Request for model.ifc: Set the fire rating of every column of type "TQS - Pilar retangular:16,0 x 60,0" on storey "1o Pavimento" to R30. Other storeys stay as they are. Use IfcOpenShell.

First a look at what the model holds.

```python
import ifcopenshell
import ifcopenshell.util.element

model = ifcopenshell.open("model.ifc")
print(model.schema)
storey = next(s for s in model.by_type("IfcBuildingStorey") if s.Name == "1o Pavimento")
columns = [e for e in ifcopenshell.util.element.get_decomposition(storey) if e.is_a("IfcColumn")]
seen = {}
for e in columns:
    element_type = ifcopenshell.util.element.get_type(e)
    key = (element_type.Name if element_type != e and element_type else None, ifcopenshell.util.element.get_pset(e, "Pset_ColumnCommon", "FireRating"))
    seen[key] = seen.get(key, 0) + 1
for (name, value), count in sorted(seen.items(), key=str):
    print(count, "x", name, "|", value)
```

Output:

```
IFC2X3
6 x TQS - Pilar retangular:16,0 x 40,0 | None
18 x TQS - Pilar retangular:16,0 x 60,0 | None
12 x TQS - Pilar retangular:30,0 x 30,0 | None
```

```python
import ifcopenshell
import ifcopenshell.api.pset
import ifcopenshell.util.element

model = ifcopenshell.open("model.ifc")

storey = next(s for s in model.by_type("IfcBuildingStorey") if s.Name == "1o Pavimento")
columns = [e for e in ifcopenshell.util.element.get_decomposition(storey) if e.is_a("IfcColumn")]

count = 0
for e in columns:
    element_type = ifcopenshell.util.element.get_type(e)
    if element_type in (None, e) or element_type.Name != "TQS - Pilar retangular:16,0 x 60,0":
        continue
    # add_pset returns the element's existing set when there is one.
    pset = ifcopenshell.api.pset.add_pset(model, product=e, name="Pset_ColumnCommon")
    ifcopenshell.api.pset.edit_pset(model, pset=pset, properties={"FireRating": "R30"})
    count += 1

print(count, "columns updated")

model.write("model-out.ifc")
```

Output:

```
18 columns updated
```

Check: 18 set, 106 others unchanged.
